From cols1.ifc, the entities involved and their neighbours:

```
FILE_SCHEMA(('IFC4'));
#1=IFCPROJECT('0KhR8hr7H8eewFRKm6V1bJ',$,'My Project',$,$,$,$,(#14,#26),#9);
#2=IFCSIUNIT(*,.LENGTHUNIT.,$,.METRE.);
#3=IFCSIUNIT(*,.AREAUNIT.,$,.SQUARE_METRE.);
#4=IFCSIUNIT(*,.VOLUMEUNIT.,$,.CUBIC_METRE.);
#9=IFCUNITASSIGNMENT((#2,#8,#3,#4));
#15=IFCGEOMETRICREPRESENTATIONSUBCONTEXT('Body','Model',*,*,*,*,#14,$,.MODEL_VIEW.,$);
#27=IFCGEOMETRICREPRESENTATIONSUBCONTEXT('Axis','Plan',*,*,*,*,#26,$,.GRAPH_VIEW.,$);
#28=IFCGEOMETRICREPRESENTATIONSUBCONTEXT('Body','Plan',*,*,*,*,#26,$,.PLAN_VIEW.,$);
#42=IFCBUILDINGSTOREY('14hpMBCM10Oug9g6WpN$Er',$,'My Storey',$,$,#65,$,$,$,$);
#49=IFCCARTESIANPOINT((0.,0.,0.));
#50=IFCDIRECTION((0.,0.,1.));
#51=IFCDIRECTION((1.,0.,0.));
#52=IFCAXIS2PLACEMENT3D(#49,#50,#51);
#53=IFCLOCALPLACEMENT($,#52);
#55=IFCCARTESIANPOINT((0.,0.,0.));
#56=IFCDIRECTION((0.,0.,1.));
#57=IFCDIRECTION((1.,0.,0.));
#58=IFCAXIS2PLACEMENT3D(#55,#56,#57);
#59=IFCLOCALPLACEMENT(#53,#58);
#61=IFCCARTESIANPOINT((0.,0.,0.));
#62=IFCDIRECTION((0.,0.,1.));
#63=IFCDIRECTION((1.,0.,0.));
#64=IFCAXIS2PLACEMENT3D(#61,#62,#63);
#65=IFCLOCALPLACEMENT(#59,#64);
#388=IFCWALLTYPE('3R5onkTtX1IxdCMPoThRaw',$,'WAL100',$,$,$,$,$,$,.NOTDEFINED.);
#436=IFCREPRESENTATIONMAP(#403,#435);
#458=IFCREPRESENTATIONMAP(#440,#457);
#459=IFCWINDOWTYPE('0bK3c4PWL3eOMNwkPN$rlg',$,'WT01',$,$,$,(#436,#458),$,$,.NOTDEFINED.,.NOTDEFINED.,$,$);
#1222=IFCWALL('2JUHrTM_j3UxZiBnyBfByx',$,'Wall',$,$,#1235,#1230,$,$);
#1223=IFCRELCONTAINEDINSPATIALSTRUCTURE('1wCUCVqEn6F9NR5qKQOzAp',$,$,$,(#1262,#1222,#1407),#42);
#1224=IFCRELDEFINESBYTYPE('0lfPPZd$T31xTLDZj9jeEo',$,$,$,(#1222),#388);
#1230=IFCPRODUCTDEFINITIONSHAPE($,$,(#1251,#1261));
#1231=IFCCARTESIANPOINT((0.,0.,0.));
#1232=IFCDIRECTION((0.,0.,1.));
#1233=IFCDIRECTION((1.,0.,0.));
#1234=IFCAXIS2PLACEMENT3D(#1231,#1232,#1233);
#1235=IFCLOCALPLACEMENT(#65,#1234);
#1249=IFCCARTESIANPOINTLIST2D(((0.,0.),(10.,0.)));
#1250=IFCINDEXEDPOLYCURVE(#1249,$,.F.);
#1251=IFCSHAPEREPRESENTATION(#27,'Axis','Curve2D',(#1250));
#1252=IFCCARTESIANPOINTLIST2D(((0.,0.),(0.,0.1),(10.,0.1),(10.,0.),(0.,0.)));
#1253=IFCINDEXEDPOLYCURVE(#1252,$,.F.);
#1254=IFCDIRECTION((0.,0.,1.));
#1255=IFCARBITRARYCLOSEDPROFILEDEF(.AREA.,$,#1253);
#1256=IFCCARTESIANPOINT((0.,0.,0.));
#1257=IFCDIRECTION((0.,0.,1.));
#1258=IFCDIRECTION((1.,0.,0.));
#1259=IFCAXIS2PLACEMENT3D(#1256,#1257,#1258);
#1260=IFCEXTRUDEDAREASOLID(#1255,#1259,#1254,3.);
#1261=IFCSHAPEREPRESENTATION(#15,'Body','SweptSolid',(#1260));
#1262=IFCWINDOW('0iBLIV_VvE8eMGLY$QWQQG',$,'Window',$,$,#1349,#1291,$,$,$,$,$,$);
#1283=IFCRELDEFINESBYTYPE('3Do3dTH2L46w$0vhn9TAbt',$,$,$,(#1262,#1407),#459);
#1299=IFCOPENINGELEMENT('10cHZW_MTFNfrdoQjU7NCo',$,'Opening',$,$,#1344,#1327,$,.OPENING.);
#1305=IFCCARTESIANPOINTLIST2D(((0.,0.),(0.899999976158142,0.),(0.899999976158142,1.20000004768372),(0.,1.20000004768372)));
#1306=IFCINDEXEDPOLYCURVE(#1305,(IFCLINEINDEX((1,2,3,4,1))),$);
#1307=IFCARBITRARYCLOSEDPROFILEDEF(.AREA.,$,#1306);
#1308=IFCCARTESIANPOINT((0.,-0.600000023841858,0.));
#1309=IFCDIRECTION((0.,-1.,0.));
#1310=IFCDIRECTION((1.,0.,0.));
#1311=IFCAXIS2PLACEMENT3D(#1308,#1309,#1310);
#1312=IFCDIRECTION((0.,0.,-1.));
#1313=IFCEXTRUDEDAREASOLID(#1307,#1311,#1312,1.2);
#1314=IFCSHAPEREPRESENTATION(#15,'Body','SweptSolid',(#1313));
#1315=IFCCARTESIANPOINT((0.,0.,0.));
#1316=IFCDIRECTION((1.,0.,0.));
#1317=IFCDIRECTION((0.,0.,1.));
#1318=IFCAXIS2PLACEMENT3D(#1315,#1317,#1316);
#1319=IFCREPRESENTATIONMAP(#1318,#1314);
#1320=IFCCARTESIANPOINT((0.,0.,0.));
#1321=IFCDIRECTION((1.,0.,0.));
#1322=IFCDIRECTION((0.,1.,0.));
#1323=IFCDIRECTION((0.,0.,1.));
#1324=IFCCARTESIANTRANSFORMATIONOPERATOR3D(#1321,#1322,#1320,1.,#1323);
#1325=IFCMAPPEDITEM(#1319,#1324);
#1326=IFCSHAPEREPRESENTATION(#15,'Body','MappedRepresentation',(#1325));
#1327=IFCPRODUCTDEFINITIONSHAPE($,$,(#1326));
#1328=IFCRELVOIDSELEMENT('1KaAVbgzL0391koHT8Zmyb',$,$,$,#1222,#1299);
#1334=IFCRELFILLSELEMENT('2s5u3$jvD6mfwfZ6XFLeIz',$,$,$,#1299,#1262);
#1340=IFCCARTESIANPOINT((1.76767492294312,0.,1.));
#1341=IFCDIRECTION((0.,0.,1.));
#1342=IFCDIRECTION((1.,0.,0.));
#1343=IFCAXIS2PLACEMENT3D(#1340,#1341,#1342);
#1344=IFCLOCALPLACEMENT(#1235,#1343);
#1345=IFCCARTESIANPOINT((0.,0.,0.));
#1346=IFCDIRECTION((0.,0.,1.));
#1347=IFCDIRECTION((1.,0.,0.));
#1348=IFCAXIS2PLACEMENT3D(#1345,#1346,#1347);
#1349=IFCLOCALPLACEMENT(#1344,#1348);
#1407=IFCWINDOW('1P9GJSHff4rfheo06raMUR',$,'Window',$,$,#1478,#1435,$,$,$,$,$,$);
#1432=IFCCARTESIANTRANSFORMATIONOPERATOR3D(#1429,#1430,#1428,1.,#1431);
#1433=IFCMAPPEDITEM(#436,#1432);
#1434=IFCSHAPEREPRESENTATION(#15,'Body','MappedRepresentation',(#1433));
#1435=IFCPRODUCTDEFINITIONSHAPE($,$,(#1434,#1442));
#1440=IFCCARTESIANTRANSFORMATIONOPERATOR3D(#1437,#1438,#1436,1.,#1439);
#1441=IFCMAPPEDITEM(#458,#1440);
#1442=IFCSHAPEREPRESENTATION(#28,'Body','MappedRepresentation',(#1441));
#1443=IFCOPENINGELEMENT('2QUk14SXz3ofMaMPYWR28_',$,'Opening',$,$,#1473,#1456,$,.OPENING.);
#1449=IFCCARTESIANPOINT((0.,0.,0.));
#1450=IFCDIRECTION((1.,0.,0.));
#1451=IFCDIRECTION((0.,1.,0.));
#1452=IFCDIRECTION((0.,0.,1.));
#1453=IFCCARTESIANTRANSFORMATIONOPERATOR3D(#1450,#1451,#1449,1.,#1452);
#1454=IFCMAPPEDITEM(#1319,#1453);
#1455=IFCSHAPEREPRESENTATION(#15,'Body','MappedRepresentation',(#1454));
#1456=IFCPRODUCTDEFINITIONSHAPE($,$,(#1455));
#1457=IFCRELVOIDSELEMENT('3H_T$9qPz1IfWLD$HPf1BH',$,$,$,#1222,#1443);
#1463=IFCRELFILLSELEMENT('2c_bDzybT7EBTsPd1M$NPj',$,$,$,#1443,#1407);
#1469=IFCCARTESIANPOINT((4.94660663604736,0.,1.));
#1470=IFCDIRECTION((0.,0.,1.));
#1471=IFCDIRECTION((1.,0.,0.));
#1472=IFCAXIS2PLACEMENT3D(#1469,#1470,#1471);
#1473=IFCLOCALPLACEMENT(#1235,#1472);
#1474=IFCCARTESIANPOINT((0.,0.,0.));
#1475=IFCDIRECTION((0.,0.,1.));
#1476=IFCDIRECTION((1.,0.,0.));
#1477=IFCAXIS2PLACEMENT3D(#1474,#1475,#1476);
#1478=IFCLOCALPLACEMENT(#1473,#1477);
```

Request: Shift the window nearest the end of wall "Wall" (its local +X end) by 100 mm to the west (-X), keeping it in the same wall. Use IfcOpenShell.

```python
import ifcopenshell
import ifcopenshell.api.geometry
import ifcopenshell.util.placement

model = ifcopenshell.open("cols1.ifc")

window = model.by_id(1407)
opening = window.FillsVoids[0].RelatingOpeningElement
wall = opening.VoidsElements[0].RelatingBuildingElement

wall_matrix = ifcopenshell.util.placement.get_local_placement(wall.ObjectPlacement)
shift = wall_matrix[:3, 0] * -0.1
before = ifcopenshell.util.placement.get_local_placement(window.ObjectPlacement)[:3, 3].copy()

# The window is placed relative to its opening, so it follows when the opening moves.
matrix = ifcopenshell.util.placement.get_local_placement(opening.ObjectPlacement)
matrix[:3, 3] += shift
ifcopenshell.api.geometry.edit_object_placement(
    model, product=opening, matrix=matrix, is_si=False, should_transform_children=True
)

after = ifcopenshell.util.placement.get_local_placement(window.ObjectPlacement)[:3, 3]
print("window moved by", (after - before).round(3) + 0.0)

model.write("cols1_v2.ifc")
```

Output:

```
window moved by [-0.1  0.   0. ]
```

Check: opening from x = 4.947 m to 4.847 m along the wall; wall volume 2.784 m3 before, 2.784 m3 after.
